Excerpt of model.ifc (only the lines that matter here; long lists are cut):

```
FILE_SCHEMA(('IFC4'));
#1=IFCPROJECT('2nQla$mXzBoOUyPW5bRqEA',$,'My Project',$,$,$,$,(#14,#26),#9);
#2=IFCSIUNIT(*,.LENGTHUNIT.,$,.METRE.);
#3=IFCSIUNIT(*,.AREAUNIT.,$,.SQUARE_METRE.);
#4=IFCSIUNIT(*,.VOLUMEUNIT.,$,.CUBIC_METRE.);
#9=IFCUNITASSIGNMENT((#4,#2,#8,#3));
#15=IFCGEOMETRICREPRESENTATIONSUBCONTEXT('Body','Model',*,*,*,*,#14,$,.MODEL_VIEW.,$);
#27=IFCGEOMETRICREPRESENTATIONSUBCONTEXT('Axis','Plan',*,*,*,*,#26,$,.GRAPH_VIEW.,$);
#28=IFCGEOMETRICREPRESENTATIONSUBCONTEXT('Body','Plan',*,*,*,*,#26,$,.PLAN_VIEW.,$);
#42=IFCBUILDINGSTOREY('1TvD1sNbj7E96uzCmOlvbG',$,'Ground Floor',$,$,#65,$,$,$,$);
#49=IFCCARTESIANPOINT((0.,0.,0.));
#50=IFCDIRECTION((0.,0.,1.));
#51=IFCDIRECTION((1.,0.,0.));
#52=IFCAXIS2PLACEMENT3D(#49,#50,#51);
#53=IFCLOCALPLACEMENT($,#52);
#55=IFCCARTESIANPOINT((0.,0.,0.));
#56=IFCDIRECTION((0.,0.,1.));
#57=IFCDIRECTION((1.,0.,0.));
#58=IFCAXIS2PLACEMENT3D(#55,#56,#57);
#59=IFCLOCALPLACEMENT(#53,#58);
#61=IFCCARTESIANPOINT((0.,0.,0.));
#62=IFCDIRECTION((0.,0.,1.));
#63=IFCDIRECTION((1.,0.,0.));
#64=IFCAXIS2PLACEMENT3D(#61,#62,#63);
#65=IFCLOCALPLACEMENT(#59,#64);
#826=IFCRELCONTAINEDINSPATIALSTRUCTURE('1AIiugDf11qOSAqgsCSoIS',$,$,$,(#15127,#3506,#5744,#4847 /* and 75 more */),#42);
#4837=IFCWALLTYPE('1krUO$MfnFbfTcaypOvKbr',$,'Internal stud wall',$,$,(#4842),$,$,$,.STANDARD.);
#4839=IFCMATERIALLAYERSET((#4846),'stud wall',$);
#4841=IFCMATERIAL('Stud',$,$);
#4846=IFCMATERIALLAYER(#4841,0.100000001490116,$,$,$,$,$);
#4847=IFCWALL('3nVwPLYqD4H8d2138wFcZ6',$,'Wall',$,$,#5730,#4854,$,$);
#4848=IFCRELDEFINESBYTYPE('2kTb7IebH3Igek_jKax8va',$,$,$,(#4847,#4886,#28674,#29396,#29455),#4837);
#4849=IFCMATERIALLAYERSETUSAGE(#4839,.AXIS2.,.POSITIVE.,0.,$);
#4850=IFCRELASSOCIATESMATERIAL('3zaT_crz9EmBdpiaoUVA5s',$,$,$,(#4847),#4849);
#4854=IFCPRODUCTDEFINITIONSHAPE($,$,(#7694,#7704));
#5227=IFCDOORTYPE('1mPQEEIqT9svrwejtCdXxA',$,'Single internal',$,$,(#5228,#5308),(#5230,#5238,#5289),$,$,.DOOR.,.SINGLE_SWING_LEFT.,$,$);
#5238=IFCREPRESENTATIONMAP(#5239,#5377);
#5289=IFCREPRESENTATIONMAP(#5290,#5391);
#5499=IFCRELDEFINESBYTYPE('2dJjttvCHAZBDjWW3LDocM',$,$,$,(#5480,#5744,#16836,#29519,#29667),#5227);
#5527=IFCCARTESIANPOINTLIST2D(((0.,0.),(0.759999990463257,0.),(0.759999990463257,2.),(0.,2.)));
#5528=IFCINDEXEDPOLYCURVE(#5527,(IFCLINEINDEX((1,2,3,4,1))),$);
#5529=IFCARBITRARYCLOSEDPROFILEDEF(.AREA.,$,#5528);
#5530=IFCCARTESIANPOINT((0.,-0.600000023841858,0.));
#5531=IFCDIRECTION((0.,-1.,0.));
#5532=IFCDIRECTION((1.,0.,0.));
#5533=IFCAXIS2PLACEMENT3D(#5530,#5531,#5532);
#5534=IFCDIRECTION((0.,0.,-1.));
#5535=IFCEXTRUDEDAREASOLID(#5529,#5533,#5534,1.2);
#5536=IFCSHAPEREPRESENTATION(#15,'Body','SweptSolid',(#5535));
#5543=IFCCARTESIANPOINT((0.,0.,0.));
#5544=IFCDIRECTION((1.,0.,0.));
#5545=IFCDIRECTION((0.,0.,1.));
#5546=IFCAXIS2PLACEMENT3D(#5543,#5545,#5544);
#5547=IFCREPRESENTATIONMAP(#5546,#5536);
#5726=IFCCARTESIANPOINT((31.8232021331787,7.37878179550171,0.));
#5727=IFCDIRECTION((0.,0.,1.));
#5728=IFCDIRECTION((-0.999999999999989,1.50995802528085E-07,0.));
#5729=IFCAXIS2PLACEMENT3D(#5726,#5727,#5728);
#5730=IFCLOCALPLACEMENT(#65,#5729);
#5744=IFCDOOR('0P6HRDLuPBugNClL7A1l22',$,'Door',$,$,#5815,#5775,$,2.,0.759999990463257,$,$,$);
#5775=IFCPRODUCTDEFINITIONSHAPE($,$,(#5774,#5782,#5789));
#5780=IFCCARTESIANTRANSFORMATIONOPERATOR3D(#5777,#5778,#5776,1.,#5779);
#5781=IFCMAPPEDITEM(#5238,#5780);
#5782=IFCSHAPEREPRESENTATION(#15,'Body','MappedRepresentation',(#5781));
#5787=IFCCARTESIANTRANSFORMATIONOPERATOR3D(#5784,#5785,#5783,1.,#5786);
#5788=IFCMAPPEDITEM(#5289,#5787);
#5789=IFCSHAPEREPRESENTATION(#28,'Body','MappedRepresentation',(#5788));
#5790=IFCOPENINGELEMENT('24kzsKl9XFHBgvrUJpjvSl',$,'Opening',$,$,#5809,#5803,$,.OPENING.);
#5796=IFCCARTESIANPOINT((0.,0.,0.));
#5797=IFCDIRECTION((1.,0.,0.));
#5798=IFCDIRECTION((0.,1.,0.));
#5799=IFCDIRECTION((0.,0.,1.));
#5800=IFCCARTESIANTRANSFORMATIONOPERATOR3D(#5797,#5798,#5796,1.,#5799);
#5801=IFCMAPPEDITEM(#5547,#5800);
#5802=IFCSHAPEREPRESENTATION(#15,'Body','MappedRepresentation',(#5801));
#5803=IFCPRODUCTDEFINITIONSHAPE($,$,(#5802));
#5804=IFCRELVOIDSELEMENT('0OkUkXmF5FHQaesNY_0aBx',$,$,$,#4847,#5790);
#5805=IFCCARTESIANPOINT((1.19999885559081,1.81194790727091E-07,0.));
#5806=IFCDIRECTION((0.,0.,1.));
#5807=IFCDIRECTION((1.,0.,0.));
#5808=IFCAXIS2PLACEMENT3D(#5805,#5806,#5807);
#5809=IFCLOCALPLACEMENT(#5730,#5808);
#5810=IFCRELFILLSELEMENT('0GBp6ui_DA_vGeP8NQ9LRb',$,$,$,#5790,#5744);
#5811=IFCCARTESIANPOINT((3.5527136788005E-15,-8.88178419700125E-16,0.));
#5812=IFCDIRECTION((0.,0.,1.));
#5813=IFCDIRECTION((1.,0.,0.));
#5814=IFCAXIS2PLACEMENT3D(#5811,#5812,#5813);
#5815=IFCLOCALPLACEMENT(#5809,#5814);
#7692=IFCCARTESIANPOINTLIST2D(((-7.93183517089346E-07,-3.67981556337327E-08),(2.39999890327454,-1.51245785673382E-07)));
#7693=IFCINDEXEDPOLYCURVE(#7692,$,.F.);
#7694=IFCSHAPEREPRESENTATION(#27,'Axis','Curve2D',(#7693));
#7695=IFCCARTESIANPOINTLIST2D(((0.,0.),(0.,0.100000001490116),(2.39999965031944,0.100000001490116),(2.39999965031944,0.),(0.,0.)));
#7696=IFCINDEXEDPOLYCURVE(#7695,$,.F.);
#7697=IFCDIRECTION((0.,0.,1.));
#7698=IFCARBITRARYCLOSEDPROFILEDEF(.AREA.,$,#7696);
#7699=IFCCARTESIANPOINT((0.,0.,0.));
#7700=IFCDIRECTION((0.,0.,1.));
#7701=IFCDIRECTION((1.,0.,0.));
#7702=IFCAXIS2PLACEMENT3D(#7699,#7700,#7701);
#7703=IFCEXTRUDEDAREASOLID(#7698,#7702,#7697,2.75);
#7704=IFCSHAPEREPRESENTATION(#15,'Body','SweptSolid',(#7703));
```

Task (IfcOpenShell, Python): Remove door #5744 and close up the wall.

```python
import ifcopenshell
import ifcopenshell.api.feature
import ifcopenshell.api.root
import ifcopenshell.geom
import ifcopenshell.util.shape

model = ifcopenshell.open("model.ifc")
settings = ifcopenshell.geom.settings()


def volume(element):
    """Net volume in cubic metres, openings subtracted."""
    shape = ifcopenshell.geom.create_shape(settings, element)
    return ifcopenshell.util.shape.get_volume(shape.geometry)


door = model.by_guid("0P6HRDLuPBugNClL7A1l22")
opening = door.FillsVoids[0].RelatingOpeningElement
wall = opening.VoidsElements[0].RelatingBuildingElement
before = volume(wall)

ifcopenshell.api.root.remove_product(model, product=door)
ifcopenshell.api.feature.remove_feature(model, feature=opening)

after = volume(wall)

print(f"wall volume {before:.3f} -> {after:.3f} m3")

model.write("model_edited.ifc")
```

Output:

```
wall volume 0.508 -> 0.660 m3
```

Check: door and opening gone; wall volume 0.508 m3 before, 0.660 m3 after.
